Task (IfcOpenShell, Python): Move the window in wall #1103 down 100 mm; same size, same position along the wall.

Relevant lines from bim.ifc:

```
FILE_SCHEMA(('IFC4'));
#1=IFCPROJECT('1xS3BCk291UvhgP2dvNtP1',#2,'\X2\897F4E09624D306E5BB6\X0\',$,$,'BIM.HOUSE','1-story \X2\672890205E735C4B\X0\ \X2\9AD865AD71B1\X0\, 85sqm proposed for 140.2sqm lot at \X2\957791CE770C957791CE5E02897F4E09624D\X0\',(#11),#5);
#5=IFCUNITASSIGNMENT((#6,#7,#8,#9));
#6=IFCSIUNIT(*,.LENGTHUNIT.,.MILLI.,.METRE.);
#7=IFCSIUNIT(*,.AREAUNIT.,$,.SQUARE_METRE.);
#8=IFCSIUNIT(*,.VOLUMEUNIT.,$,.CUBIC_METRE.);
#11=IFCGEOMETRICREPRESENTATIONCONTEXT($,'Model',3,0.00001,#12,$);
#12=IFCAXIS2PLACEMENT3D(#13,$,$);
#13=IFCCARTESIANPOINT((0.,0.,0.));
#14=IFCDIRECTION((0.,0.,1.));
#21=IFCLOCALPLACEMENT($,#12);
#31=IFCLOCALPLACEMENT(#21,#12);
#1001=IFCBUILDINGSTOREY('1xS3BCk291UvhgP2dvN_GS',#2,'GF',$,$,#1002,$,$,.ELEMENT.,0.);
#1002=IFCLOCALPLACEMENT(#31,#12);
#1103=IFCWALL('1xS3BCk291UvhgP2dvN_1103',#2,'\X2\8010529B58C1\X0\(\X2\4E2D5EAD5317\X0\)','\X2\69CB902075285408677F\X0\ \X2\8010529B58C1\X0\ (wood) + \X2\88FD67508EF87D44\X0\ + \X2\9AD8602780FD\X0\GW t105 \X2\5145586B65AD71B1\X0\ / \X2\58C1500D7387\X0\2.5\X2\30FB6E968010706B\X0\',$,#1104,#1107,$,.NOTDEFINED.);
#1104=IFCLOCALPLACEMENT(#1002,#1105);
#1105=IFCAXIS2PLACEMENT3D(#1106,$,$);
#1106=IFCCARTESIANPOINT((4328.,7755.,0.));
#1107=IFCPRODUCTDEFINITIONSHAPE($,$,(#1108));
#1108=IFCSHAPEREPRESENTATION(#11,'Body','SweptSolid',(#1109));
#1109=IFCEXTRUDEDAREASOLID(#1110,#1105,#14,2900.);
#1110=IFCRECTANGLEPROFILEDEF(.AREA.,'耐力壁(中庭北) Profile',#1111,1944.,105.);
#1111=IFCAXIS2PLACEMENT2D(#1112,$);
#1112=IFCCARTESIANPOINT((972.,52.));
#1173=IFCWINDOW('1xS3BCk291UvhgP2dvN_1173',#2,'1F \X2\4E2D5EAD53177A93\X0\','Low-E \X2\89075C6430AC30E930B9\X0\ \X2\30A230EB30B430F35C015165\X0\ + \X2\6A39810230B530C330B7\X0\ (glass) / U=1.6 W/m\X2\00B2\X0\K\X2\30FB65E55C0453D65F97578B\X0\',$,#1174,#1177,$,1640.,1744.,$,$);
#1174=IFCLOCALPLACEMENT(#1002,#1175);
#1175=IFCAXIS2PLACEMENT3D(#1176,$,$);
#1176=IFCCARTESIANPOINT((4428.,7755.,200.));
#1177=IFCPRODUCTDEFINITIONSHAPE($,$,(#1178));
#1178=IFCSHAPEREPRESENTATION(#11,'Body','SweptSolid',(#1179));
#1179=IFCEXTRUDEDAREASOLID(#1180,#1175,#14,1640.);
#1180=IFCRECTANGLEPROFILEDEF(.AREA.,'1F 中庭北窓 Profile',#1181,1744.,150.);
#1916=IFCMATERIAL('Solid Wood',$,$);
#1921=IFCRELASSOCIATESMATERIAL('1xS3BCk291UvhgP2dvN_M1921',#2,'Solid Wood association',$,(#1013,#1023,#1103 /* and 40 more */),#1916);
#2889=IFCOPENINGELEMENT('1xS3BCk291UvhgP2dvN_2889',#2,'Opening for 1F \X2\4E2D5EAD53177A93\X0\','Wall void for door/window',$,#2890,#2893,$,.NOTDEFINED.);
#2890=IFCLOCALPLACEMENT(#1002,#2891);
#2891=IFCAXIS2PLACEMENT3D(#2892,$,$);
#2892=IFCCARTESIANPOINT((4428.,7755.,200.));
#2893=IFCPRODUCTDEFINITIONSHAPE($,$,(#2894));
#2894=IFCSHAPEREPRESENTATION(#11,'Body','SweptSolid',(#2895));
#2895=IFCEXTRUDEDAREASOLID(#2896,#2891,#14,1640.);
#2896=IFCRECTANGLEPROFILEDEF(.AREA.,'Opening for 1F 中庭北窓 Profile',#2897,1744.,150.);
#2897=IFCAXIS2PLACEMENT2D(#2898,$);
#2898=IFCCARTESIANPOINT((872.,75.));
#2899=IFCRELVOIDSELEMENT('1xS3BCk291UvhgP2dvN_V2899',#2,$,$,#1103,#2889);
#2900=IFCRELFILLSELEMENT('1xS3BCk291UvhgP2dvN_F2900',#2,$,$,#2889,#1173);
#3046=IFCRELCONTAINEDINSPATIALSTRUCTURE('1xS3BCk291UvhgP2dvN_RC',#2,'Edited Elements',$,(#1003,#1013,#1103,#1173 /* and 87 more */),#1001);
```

```python
import numpy as np
import ifcopenshell
import ifcopenshell.api.geometry
import ifcopenshell.util.placement
import ifcopenshell.util.unit

model = ifcopenshell.open("bim.ifc")
unit_scale = ifcopenshell.util.unit.calculate_unit_scale(model)

window = model.by_id(1173)
opening = window.FillsVoids[0].RelatingOpeningElement
dz = -0.1 / unit_scale

shift = np.array([0.0, 0.0, dz])
# The window is not placed relative to its opening, so move both.
for product in (opening, window):
    matrix = ifcopenshell.util.placement.get_local_placement(product.ObjectPlacement)
    matrix[:3, 3] += shift
    ifcopenshell.api.geometry.edit_object_placement(model, product=product, matrix=matrix, is_si=False)

print(f"moved by {dz * unit_scale:+.3f} m")

model.write("bim_updated.ifc")
```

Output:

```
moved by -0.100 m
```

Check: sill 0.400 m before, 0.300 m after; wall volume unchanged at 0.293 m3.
